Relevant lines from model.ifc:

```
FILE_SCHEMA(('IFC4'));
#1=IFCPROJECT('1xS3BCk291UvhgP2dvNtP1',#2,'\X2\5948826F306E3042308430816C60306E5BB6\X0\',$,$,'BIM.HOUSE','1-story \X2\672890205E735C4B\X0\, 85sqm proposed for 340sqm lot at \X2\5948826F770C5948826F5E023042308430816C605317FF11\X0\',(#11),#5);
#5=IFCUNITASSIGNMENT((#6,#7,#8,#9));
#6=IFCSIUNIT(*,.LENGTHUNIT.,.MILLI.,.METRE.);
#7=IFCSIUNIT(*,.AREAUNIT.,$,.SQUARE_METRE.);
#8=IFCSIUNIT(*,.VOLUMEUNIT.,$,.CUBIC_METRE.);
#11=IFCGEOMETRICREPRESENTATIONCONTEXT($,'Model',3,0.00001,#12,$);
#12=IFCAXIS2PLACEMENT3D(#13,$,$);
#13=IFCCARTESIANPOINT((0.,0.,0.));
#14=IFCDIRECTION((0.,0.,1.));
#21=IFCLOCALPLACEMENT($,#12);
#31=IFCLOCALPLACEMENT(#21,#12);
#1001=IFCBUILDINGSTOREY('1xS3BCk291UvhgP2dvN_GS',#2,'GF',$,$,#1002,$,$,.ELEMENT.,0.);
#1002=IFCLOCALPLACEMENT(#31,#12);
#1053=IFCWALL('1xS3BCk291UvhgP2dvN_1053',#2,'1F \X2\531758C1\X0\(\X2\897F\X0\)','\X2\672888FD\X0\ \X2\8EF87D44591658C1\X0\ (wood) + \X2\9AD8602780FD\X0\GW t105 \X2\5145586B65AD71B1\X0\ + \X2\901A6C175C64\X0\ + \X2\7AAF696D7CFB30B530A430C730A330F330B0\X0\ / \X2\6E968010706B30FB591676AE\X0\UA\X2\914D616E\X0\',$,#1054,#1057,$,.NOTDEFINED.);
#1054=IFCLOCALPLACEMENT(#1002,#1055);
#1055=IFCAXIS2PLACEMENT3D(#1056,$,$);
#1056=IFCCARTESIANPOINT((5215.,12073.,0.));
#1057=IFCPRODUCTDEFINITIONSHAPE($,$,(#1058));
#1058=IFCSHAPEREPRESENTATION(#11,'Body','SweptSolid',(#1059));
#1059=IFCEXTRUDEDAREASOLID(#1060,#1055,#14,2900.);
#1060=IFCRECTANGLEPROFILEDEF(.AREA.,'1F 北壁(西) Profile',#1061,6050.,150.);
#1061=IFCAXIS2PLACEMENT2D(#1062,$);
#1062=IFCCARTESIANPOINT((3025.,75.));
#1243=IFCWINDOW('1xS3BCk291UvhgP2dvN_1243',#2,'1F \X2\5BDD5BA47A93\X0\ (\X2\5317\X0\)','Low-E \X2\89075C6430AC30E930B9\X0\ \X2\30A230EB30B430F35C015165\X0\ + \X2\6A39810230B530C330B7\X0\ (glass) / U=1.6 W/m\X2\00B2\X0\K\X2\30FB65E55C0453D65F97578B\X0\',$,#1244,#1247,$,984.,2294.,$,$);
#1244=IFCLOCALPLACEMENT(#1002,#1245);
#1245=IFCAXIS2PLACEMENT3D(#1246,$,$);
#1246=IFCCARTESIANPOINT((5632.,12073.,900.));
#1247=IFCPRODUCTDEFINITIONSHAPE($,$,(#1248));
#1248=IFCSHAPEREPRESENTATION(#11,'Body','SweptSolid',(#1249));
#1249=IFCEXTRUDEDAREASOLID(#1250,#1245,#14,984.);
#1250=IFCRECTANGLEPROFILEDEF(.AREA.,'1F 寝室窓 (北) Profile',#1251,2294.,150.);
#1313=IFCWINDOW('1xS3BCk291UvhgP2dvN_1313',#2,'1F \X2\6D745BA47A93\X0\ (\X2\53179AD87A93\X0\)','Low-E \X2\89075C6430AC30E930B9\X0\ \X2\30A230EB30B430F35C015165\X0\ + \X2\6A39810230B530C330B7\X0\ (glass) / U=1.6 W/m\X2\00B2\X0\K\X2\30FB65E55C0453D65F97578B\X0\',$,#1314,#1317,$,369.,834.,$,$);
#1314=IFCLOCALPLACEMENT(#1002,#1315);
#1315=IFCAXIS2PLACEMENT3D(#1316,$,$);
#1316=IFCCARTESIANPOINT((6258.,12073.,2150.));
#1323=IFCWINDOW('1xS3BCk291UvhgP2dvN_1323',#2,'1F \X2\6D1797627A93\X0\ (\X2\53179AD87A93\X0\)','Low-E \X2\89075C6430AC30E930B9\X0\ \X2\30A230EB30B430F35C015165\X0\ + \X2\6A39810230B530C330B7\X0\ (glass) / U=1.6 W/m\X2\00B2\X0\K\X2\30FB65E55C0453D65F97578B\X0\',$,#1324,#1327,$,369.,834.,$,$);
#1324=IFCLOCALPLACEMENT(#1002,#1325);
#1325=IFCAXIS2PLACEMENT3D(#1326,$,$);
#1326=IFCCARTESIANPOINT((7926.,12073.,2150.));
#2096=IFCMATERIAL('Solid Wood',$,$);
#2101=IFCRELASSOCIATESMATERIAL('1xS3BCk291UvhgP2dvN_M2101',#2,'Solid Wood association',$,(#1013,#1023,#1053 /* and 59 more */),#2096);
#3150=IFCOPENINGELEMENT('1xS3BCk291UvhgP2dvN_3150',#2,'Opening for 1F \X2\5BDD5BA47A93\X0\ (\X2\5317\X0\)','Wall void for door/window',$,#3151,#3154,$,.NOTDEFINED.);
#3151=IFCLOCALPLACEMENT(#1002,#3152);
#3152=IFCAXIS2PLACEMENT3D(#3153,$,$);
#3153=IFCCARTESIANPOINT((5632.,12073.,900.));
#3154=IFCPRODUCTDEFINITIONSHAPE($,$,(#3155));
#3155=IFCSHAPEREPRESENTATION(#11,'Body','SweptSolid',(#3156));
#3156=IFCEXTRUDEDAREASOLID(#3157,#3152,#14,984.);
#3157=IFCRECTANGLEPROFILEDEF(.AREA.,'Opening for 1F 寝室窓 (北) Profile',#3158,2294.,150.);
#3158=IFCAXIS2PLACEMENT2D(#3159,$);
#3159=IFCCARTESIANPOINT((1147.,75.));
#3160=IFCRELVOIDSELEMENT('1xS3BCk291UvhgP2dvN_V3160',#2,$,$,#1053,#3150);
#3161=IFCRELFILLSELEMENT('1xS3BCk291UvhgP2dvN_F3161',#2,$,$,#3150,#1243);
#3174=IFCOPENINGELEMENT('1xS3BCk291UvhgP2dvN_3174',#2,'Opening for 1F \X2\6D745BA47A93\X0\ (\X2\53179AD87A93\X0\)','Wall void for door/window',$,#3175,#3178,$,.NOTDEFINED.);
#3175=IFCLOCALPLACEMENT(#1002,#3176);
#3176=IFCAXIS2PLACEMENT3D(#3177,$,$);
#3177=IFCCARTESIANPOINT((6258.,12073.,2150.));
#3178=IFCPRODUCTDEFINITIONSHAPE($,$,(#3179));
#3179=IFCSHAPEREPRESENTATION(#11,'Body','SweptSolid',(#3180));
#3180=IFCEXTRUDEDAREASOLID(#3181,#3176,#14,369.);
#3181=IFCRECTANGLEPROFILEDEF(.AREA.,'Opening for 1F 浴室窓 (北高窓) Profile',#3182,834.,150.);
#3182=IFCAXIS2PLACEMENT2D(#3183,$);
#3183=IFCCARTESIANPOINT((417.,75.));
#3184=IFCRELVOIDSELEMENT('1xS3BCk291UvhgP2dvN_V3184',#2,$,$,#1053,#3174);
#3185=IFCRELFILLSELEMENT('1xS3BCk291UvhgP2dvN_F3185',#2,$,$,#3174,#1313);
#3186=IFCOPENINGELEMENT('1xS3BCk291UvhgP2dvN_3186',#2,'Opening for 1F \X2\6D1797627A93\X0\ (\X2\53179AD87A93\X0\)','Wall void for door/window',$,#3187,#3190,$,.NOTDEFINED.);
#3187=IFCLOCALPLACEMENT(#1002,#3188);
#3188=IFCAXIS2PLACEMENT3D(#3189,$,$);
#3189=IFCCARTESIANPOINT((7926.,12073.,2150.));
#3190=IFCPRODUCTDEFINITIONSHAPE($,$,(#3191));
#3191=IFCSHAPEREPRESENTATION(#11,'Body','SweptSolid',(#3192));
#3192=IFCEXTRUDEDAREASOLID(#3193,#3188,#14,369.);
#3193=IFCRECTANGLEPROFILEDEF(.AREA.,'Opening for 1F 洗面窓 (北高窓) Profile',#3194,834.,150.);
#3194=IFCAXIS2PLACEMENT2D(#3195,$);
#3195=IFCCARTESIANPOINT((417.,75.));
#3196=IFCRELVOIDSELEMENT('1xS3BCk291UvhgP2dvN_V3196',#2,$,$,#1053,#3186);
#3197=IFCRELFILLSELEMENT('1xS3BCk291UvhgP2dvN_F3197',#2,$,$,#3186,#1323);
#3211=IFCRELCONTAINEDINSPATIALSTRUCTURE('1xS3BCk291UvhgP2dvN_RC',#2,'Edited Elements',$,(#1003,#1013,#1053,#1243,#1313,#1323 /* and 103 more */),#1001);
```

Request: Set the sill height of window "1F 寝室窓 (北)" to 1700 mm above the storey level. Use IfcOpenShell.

```python
import numpy as np
import ifcopenshell
import ifcopenshell.api.geometry
import ifcopenshell.geom
import ifcopenshell.util.element
import ifcopenshell.util.placement
import ifcopenshell.util.shape
import ifcopenshell.util.unit

model = ifcopenshell.open("model.ifc")
unit_scale = ifcopenshell.util.unit.calculate_unit_scale(model)

window = model.by_guid("1xS3BCk291UvhgP2dvN_1243")
opening = window.FillsVoids[0].RelatingOpeningElement
storey = ifcopenshell.util.element.get_container(window, ifc_class="IfcBuildingStorey")
level = ifcopenshell.util.placement.get_local_placement(storey.ObjectPlacement)[2, 3]

# The opening's origin need not be at the sill, so measure its lowest point.
shape = ifcopenshell.geom.create_shape(ifcopenshell.geom.settings(), opening)
bottom = ifcopenshell.util.shape.get_shape_bottom_elevation(shape, shape.geometry) / unit_scale
dz = level + 1700.0 - bottom

shift = np.array([0.0, 0.0, dz])
# The window is not placed relative to its opening, so move both.
for product in (opening, window):
    matrix = ifcopenshell.util.placement.get_local_placement(product.ObjectPlacement)
    matrix[:3, 3] += shift
    ifcopenshell.api.geometry.edit_object_placement(model, product=product, matrix=matrix, is_si=False)

print(f"moved by {dz * unit_scale:+.3f} m")

model.write("model_v2.ifc")
```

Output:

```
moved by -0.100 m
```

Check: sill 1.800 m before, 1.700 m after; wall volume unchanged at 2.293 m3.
